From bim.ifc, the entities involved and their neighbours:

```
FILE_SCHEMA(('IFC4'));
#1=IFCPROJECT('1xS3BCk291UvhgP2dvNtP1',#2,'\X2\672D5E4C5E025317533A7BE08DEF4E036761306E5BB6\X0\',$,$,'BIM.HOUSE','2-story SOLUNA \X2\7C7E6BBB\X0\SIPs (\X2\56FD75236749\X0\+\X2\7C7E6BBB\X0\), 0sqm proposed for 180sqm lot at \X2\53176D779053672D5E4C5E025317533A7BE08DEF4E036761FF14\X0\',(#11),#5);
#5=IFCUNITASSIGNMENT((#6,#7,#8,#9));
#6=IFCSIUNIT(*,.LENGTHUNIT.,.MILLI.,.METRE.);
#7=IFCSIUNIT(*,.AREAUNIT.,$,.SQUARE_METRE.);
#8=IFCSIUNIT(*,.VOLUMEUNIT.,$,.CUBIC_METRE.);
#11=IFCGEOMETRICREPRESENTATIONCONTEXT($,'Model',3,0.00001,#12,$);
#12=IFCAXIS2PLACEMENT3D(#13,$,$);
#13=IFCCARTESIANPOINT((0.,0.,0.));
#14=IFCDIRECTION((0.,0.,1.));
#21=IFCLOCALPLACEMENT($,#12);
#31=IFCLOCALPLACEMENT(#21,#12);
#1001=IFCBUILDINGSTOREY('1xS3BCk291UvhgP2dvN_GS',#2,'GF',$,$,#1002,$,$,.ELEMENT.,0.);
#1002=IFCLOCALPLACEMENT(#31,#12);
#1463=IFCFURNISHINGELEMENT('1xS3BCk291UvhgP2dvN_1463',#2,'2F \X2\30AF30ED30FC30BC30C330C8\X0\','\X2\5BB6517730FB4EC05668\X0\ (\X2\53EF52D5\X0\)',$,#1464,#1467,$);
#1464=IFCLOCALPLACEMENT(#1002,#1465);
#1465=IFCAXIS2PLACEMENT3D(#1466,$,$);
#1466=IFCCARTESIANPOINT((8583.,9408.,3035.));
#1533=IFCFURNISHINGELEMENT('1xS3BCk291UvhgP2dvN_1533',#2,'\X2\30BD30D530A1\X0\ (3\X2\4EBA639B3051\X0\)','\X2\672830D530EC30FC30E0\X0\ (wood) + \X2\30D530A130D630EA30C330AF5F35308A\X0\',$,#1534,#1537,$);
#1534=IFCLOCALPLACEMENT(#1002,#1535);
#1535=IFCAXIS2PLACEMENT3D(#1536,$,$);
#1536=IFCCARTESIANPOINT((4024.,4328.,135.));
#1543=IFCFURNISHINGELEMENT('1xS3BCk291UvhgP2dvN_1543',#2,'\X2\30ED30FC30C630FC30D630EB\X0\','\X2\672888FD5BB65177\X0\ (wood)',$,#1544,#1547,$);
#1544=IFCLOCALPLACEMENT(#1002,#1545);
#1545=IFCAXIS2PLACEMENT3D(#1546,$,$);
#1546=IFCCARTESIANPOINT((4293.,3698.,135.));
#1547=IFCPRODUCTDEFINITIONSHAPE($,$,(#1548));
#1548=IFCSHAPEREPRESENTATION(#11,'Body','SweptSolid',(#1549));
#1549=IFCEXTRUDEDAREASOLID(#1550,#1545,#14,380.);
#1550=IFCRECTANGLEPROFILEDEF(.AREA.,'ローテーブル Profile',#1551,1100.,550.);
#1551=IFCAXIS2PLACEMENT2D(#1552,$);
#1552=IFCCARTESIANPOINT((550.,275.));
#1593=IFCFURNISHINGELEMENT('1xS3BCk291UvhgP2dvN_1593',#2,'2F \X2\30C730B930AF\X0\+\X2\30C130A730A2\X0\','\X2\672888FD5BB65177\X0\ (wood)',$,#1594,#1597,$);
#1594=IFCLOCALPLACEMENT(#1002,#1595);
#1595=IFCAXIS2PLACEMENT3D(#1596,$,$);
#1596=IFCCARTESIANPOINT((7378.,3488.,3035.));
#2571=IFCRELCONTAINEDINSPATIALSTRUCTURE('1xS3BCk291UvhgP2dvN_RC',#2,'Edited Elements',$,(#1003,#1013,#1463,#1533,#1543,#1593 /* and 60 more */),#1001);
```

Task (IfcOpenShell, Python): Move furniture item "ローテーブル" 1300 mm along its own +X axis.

```python
import ifcopenshell
import ifcopenshell.api.geometry
import ifcopenshell.util.placement

model = ifcopenshell.open("bim.ifc")

item = model.by_guid("1xS3BCk291UvhgP2dvN_1543")
matrix = ifcopenshell.util.placement.get_local_placement(item.ObjectPlacement)
matrix[:3, 3] += matrix[:3, 0] * 1300.0
ifcopenshell.api.geometry.edit_object_placement(model, product=item, matrix=matrix, is_si=False)

print(ifcopenshell.util.placement.get_local_placement(item.ObjectPlacement).round(3) + 0.0)

model.write("bim_updated.ifc")
```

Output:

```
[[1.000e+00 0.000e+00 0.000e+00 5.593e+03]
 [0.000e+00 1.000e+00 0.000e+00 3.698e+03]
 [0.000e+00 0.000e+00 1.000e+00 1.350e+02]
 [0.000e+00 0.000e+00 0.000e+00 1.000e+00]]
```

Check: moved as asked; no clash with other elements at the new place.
